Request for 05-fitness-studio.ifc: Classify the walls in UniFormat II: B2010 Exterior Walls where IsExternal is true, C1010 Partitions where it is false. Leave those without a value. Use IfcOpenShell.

First a look at what the model holds.

```python
import ifcopenshell
import ifcopenshell.util.element

model = ifcopenshell.open("05-fitness-studio.ifc")
print(model.schema)
print("classifications:", [c.Name for c in model.by_type("IfcClassification")])
values = [ifcopenshell.util.element.get_pset(e, "Pset_WallCommon", "IsExternal") for e in model.by_type("IfcWall")]
for value in (True, False, None):
    print("IsExternal", value, values.count(value))
```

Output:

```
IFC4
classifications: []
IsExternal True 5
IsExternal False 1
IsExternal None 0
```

```python
import ifcopenshell
import ifcopenshell.api.classification
import ifcopenshell.util.element

model = ifcopenshell.open("05-fitness-studio.ifc")

system = ifcopenshell.api.classification.add_classification(model, classification="UniFormat II")

walls = model.by_type("IfcWall")
external = {e: ifcopenshell.util.element.get_pset(e, "Pset_WallCommon", "IsExternal") for e in walls}
for flag, code, name in ((True, "B2010", "Exterior Walls"), (False, "C1010", "Partitions")):
    products = [e for e in walls if external[e] is flag]
    ifcopenshell.api.classification.add_reference(
        model, products=products, classification=system, identification=code, name=name
    )
    print(code, len(products))

model.write("05-fitness-studio_v2.ifc")
```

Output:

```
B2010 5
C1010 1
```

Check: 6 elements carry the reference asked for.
